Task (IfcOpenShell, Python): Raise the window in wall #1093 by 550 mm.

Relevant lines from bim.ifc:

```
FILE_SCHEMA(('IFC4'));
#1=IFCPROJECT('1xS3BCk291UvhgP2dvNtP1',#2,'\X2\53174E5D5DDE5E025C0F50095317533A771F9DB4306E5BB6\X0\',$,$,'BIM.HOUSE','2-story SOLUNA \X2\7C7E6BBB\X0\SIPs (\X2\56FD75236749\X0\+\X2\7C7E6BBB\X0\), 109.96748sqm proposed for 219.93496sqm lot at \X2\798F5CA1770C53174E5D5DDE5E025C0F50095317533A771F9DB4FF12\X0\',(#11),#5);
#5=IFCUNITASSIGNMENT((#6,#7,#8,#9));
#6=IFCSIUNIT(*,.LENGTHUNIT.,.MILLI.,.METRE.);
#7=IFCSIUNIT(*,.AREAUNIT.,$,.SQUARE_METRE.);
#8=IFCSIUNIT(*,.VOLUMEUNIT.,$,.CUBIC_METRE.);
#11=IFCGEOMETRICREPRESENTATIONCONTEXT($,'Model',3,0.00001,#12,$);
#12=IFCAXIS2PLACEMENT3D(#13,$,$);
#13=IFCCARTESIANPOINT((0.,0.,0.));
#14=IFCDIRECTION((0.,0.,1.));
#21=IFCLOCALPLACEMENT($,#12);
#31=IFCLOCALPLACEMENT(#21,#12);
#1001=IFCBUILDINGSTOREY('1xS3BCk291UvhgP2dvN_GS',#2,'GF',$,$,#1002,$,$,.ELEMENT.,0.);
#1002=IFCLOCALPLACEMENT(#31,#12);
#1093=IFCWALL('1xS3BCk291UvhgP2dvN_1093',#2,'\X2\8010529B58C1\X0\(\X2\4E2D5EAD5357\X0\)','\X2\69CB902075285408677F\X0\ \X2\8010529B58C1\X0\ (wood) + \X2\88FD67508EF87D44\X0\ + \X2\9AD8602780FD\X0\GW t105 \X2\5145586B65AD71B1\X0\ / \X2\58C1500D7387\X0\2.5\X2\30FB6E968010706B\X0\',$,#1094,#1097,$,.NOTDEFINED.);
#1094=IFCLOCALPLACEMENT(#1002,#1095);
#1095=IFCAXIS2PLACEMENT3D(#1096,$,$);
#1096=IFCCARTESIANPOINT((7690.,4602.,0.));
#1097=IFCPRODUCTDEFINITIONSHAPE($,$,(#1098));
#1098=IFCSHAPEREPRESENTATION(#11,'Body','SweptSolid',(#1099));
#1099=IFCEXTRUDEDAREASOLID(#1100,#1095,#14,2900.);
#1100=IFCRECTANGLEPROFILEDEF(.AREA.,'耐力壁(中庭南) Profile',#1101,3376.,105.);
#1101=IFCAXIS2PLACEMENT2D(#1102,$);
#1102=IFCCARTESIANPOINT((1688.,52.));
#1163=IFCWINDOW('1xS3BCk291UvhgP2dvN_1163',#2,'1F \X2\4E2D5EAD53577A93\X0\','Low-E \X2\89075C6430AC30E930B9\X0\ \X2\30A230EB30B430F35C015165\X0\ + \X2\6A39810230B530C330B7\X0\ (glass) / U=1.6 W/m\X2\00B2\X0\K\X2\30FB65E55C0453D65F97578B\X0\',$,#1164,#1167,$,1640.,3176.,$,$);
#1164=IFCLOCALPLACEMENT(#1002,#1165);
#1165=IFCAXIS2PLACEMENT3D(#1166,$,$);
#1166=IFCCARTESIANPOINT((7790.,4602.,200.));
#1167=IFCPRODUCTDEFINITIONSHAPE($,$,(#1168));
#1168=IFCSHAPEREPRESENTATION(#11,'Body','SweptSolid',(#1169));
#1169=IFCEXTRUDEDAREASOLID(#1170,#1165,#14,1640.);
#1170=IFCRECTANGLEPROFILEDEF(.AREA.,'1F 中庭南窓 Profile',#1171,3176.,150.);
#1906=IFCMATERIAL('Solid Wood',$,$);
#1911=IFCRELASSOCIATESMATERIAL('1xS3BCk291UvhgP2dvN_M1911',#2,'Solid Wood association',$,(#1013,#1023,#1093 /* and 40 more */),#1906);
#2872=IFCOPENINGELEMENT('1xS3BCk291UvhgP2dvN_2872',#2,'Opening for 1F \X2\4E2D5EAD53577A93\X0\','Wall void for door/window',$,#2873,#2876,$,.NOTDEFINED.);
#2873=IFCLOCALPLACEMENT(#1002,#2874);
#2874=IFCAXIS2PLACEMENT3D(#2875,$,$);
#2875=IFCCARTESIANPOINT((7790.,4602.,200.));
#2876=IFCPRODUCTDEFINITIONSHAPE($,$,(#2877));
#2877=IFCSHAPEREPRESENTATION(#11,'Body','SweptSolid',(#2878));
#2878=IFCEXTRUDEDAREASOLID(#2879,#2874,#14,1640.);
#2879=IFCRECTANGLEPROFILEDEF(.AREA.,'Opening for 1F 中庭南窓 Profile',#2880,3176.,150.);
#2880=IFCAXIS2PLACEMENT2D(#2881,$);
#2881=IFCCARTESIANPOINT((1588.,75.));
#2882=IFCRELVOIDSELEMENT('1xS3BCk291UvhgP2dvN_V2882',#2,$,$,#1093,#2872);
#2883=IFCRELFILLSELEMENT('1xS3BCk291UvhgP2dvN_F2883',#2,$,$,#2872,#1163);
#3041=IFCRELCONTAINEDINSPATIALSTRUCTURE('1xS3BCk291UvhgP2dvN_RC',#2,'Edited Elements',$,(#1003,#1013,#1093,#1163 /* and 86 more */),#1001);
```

```python
import numpy as np
import ifcopenshell
import ifcopenshell.api.geometry
import ifcopenshell.util.placement
import ifcopenshell.util.unit

model = ifcopenshell.open("bim.ifc")
unit_scale = ifcopenshell.util.unit.calculate_unit_scale(model)

window = model.by_guid("1xS3BCk291UvhgP2dvN_1163")
opening = window.FillsVoids[0].RelatingOpeningElement
dz = 0.55 / unit_scale

shift = np.array([0.0, 0.0, dz])
# The window is not placed relative to its opening, so move both.
for product in (opening, window):
    matrix = ifcopenshell.util.placement.get_local_placement(product.ObjectPlacement)
    matrix[:3, 3] += shift
    ifcopenshell.api.geometry.edit_object_placement(model, product=product, matrix=matrix, is_si=False)

print(f"moved by {dz * unit_scale:+.3f} m")

model.write("bim_rev.ifc")
```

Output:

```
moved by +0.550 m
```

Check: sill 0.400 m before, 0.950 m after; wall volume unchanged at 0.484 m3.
